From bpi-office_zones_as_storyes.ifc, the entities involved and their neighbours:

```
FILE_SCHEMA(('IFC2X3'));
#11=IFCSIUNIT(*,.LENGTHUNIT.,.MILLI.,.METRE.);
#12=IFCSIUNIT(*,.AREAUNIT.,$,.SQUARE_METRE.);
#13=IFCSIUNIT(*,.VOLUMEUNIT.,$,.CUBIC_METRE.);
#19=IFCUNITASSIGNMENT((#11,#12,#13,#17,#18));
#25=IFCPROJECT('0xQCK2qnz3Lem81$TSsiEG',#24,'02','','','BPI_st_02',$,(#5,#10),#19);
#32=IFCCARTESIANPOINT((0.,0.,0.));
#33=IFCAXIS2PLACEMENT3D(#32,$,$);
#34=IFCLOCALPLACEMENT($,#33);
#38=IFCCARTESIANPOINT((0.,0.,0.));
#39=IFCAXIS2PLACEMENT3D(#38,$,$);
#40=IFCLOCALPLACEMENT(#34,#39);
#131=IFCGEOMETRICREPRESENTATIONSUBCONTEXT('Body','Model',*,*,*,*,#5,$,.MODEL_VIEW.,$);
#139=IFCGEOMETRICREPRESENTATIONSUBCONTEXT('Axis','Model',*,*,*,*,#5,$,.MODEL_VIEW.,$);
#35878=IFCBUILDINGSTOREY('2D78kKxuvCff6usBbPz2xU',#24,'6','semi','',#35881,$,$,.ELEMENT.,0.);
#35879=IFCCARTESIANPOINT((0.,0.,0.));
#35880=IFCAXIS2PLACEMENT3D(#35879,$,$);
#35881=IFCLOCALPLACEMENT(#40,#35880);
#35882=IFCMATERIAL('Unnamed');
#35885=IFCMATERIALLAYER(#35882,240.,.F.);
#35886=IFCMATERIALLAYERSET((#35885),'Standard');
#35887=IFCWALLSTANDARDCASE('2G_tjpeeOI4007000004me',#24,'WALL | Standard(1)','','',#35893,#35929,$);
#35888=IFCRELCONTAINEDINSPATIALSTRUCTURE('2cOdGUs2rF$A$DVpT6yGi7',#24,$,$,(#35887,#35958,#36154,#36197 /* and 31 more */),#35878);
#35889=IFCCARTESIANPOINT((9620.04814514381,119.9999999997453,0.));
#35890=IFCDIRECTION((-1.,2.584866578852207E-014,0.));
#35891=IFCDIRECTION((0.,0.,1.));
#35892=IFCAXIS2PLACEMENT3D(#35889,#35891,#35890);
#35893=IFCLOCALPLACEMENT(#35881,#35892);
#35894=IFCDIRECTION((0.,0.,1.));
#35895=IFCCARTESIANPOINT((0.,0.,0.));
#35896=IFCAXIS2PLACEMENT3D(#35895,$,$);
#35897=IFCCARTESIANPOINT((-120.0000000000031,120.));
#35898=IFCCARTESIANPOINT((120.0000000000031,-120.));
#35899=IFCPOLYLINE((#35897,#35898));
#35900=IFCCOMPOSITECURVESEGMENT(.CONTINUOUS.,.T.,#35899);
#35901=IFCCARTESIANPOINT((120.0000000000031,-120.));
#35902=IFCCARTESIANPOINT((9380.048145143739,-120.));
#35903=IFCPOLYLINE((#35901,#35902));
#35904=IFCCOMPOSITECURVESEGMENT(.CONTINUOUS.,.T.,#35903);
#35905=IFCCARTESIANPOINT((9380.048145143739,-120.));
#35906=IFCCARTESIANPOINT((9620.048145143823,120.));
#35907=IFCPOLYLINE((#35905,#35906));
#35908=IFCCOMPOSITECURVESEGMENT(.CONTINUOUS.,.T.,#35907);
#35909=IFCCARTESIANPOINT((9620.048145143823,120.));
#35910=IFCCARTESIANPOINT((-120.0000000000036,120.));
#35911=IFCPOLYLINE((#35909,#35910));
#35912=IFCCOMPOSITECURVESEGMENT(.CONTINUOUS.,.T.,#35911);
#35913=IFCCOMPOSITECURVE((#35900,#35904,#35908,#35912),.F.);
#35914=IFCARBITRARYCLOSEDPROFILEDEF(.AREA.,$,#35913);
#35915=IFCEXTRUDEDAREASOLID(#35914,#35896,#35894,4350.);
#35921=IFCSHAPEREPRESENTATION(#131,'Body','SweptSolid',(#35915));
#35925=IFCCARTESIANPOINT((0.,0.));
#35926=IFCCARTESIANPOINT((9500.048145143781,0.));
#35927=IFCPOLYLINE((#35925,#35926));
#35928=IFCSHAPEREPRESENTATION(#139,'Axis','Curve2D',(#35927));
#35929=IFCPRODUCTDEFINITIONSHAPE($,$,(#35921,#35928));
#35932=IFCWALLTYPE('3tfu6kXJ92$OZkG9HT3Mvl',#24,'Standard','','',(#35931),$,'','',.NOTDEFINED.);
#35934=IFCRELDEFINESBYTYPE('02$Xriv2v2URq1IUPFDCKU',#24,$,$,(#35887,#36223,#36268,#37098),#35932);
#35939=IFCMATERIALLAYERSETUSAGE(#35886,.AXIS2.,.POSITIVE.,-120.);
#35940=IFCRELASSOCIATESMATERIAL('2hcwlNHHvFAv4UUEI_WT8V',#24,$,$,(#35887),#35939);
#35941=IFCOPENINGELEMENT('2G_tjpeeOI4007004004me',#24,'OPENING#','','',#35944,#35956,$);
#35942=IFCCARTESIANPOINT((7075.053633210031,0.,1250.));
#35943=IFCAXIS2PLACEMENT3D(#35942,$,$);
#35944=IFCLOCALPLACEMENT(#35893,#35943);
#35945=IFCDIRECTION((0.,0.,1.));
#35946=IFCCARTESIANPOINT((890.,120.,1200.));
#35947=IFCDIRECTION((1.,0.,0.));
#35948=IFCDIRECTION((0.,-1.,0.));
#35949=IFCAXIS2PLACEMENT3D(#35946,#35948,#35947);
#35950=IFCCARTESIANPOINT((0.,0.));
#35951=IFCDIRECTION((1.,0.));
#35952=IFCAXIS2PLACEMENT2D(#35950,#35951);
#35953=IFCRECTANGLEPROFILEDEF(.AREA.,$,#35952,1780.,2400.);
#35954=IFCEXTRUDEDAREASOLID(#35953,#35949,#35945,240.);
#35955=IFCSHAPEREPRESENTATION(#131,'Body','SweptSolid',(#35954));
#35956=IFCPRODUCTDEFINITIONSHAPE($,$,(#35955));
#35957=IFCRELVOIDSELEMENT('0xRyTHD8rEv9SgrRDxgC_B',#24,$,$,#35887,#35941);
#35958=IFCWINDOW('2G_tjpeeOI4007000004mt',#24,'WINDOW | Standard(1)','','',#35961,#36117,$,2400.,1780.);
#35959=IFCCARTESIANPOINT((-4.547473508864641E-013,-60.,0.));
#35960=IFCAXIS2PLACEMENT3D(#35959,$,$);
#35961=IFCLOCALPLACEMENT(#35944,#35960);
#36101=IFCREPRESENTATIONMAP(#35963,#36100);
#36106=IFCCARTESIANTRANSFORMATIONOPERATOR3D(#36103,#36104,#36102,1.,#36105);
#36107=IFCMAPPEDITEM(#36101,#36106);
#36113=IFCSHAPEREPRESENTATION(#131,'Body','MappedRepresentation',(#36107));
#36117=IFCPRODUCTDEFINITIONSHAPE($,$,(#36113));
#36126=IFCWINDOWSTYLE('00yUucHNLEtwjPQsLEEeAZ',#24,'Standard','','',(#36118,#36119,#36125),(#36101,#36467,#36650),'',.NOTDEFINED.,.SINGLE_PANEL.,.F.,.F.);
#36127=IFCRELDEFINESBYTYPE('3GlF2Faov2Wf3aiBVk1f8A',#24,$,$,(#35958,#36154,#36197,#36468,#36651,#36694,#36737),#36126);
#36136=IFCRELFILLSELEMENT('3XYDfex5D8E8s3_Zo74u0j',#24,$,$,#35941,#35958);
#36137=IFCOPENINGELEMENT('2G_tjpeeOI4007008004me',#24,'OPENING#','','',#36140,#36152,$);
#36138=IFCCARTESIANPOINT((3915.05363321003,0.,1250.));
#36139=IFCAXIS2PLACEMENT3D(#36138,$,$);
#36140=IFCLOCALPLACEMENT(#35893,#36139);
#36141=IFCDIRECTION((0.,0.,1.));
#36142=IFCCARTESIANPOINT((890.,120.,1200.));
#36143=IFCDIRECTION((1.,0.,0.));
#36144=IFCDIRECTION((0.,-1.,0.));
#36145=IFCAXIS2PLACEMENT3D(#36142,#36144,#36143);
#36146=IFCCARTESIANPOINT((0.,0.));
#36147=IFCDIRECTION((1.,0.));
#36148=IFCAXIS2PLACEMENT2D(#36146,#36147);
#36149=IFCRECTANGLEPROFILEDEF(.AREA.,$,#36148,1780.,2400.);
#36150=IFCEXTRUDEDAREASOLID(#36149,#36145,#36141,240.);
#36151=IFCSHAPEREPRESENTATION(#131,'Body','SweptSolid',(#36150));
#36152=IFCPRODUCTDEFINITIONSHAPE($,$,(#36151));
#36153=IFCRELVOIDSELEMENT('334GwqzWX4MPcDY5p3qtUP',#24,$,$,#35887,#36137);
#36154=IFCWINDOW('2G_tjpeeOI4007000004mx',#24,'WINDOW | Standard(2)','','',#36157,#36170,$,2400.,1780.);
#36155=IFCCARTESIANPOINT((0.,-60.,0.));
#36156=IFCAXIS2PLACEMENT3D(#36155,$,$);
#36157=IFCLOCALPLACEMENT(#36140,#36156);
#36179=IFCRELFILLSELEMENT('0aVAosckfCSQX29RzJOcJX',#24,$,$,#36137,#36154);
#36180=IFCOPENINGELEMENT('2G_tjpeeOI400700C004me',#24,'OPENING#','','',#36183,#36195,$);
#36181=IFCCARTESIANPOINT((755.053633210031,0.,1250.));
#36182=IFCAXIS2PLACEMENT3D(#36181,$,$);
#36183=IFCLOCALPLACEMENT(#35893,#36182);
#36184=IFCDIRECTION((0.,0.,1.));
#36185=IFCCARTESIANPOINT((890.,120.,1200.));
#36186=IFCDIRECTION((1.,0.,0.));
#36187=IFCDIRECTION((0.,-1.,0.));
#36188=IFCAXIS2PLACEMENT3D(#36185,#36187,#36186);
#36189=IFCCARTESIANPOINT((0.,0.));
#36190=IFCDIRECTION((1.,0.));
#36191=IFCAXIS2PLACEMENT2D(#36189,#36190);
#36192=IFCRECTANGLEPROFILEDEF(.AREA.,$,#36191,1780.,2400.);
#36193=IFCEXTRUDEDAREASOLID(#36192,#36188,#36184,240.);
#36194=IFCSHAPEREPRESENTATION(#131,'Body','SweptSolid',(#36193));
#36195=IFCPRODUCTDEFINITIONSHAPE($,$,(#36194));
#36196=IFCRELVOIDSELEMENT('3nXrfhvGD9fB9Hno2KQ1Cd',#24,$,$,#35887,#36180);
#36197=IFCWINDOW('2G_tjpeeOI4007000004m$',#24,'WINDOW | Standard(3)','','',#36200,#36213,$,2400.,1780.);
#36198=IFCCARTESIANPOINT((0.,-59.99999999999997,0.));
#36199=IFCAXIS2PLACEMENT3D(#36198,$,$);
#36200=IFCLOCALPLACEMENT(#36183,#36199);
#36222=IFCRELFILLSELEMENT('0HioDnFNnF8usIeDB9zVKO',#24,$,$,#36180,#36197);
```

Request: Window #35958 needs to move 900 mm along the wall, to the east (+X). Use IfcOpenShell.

```python
import ifcopenshell
import ifcopenshell.api.geometry
import ifcopenshell.util.placement
import ifcopenshell.util.unit

model = ifcopenshell.open("bpi-office_zones_as_storyes.ifc")
unit_scale = ifcopenshell.util.unit.calculate_unit_scale(model)

window = model.by_guid("2G_tjpeeOI4007000004mt")
opening = window.FillsVoids[0].RelatingOpeningElement
wall = opening.VoidsElements[0].RelatingBuildingElement

wall_matrix = ifcopenshell.util.placement.get_local_placement(wall.ObjectPlacement)
shift = wall_matrix[:3, 0] * -0.9 / unit_scale
before = ifcopenshell.util.placement.get_local_placement(window.ObjectPlacement)[:3, 3].copy()

# The window is placed relative to its opening, so it follows when the opening moves.
matrix = ifcopenshell.util.placement.get_local_placement(opening.ObjectPlacement)
matrix[:3, 3] += shift
ifcopenshell.api.geometry.edit_object_placement(
    model, product=opening, matrix=matrix, is_si=False, should_transform_children=True
)

after = ifcopenshell.util.placement.get_local_placement(window.ObjectPlacement)[:3, 3]
print("window moved by", (after - before).round(3) + 0.0)

model.write("bpi-office_zones_as_storyes_rev.ifc")
```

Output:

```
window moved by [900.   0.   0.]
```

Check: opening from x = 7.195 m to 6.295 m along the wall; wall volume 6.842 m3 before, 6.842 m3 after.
